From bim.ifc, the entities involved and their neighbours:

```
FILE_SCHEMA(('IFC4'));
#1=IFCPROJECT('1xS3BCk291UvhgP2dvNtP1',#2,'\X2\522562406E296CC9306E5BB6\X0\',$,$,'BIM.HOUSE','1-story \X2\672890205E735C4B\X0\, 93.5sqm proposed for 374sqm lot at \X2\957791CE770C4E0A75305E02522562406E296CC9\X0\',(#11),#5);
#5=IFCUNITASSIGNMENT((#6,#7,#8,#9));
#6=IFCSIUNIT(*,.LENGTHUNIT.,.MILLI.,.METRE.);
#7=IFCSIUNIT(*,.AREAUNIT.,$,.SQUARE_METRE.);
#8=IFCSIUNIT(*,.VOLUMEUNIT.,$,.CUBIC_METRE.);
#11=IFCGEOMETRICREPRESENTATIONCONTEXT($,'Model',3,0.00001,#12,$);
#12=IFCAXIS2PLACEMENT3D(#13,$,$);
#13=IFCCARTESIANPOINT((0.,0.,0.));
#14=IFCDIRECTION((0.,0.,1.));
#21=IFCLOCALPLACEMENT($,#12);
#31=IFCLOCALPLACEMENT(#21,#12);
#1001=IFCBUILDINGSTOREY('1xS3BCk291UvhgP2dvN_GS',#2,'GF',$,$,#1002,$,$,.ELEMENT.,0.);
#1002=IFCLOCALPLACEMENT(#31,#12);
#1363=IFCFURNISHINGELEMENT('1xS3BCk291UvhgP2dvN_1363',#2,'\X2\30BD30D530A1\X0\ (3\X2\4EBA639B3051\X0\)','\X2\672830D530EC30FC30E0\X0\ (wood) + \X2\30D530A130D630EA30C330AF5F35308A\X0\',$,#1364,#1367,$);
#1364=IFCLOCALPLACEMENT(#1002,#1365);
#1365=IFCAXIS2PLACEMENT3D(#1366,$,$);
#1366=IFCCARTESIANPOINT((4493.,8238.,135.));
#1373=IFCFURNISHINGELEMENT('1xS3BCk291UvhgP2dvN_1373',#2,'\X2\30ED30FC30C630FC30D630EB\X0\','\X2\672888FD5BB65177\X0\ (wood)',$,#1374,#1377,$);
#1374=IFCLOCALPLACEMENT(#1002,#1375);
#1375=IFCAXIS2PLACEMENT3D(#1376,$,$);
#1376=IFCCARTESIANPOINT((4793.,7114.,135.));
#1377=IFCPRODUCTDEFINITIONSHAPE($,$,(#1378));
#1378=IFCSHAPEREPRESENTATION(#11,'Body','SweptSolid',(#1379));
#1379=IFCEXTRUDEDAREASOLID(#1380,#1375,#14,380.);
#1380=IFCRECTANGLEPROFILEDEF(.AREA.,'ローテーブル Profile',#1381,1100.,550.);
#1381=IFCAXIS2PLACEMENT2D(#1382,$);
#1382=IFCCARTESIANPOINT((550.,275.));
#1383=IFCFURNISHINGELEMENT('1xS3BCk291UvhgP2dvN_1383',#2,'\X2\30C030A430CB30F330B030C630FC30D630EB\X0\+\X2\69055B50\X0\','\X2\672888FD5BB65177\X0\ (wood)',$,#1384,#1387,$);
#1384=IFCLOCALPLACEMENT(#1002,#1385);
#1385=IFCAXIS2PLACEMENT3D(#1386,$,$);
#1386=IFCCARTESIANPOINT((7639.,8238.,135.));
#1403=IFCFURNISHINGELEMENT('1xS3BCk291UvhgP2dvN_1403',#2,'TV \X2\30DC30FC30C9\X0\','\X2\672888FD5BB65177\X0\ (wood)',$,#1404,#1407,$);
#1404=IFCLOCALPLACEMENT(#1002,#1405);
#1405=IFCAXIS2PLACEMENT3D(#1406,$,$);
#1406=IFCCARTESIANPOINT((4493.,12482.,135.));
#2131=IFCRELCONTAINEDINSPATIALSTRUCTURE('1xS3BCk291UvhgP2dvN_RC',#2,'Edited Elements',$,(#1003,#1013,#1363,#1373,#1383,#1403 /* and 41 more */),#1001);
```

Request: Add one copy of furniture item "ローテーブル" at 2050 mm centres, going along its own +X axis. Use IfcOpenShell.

```python
import ifcopenshell
import ifcopenshell.api.geometry
import ifcopenshell.api.root
import ifcopenshell.util.element
import ifcopenshell.util.placement
import ifcopenshell.util.unit

model = ifcopenshell.open("bim.ifc")
unit_scale = ifcopenshell.util.unit.calculate_unit_scale(model)


def reuse_history(source, copy):
    """copy_class also copies each property set's owner history, people and application; keep the originals."""
    for rel in copy.IsDefinedBy:
        if rel.is_a("IfcRelDefinesByProperties") and (history := rel.RelatingPropertyDefinition.OwnerHistory):
            rel.RelatingPropertyDefinition.OwnerHistory = source.OwnerHistory
            ifcopenshell.util.element.remove_deep2(model, history)


source = model.by_id(1373)
base = ifcopenshell.util.placement.get_local_placement(source.ObjectPlacement)
step = base[:3, 0] * 2.05 / unit_scale

for i in range(1, 2):
    copy = ifcopenshell.api.root.copy_class(model, product=source)
    copy.Representation = ifcopenshell.util.element.copy_deep(
        model, source.Representation, exclude=["IfcGeometricRepresentationContext", "IfcRepresentationMap"]
    )
    reuse_history(source, copy)
    matrix = base.copy()
    matrix[:3, 3] += i * step
    print("added at", matrix[:3, 3].round(3) + 0.0)
    ifcopenshell.api.geometry.edit_object_placement(model, product=copy, matrix=matrix, is_si=False)

model.write("bim_rev.ifc")
```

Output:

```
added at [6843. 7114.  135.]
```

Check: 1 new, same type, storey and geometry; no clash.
